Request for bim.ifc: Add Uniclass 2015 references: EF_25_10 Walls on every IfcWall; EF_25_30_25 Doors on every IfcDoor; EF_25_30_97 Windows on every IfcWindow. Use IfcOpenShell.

First a look at what the model holds.

```python
import ifcopenshell

model = ifcopenshell.open("bim.ifc")
print(model.schema)
print("classifications:", [c.Name for c in model.by_type("IfcClassification")])
for ifc_class in ("IfcDoor", "IfcRoof", "IfcStair", "IfcWall", "IfcWindow"):
    print(ifc_class, len(model.by_type(ifc_class)))
```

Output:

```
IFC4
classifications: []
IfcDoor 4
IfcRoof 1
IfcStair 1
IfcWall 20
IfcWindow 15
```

```python
import ifcopenshell
import ifcopenshell.api.classification

model = ifcopenshell.open("bim.ifc")

system = ifcopenshell.api.classification.add_classification(model, classification="Uniclass 2015")

codes = {
    "IfcWall": ("EF_25_10", "Walls"),
    "IfcDoor": ("EF_25_30_25", "Doors"),
    "IfcWindow": ("EF_25_30_97", "Windows"),
}
for ifc_class, (code, name) in codes.items():
    products = model.by_type(ifc_class)
    ifcopenshell.api.classification.add_reference(
        model, products=products, classification=system, identification=code, name=name
    )
    print(code, len(products))

model.write("bim_updated.ifc")
```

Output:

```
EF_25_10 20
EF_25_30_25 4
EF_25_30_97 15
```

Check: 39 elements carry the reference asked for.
